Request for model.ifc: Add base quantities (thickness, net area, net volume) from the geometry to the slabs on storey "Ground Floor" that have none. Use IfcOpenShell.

First a look at what the model holds.

```python
import ifcopenshell
import ifcopenshell.util.element
import ifcopenshell.util.unit

model = ifcopenshell.open("model.ifc")
print(model.schema)
for unit_type in ("LENGTHUNIT", "AREAUNIT", "VOLUMEUNIT"):
    print(unit_type, ifcopenshell.util.unit.calculate_unit_scale(model, unit_type))
storey = next(s for s in model.by_type("IfcBuildingStorey") if s.Name == "Ground Floor")
slabs = [e for e in ifcopenshell.util.element.get_decomposition(storey) if e.is_a("IfcSlab")]
for e in sorted(slabs, key=lambda e: e.id()):
    print(e.id(), e.is_a(), e.Name, list(ifcopenshell.util.element.get_psets(e, qtos_only=True)), sep=" | ")
```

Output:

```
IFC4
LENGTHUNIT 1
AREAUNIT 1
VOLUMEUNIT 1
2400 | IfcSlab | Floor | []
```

```python
import ifcopenshell
import ifcopenshell.api.pset
import ifcopenshell.geom
import ifcopenshell.util.element
import ifcopenshell.util.shape
import ifcopenshell.util.unit

model = ifcopenshell.open("model.ifc")
unit_scale = ifcopenshell.util.unit.calculate_unit_scale(model)
area_scale = ifcopenshell.util.unit.calculate_unit_scale(model, "AREAUNIT")
volume_scale = ifcopenshell.util.unit.calculate_unit_scale(model, "VOLUMEUNIT")
settings = ifcopenshell.geom.settings()

storey = next(s for s in model.by_type("IfcBuildingStorey") if s.Name == "Ground Floor")
slabs = [e for e in ifcopenshell.util.element.get_decomposition(storey) if e.is_a("IfcSlab")]

for e in sorted(slabs, key=lambda e: e.id()):
    if ifcopenshell.util.element.get_psets(e, qtos_only=True, should_inherit=False):
        continue
    # Geometry comes back in metres, in the element's own axes.
    shape = ifcopenshell.geom.create_shape(settings, e)
    values = {
        "Width": ifcopenshell.util.shape.get_z(shape.geometry) / unit_scale,
        "NetArea": ifcopenshell.util.shape.get_footprint_area(shape.geometry) / area_scale,
        "NetVolume": ifcopenshell.util.shape.get_volume(shape.geometry) / volume_scale,
    }
    qto = ifcopenshell.api.pset.add_qto(model, product=e, name="Qto_SlabBaseQuantities")
    ifcopenshell.api.pset.edit_qto(model, qto=qto, properties=values)
    print(e.id(), {k: round(v, 3) for k, v in values.items()})

model.write("model_updated.ifc")
```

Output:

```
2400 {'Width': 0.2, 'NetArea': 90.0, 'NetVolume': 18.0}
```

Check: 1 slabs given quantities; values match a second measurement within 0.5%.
